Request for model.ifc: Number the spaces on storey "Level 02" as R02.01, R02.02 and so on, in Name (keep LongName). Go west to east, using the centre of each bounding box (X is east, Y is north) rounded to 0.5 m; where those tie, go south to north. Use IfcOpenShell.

First a look at what the model holds.

```python
import ifcopenshell
import ifcopenshell.util.element
import ifcopenshell.util.placement

model = ifcopenshell.open("model.ifc")
print(model.schema)
storey = next(s for s in model.by_type("IfcBuildingStorey") if s.Name == "Level 02")
spaces = [e for e in ifcopenshell.util.element.get_decomposition(storey) if e.is_a("IfcSpace")]
for e in sorted(spaces, key=lambda e: e.id()):
    origin = ifcopenshell.util.placement.get_local_placement(e.ObjectPlacement)[:3, 3]
    print(e.id(), e.Name, e.LongName, origin.round(2) + 0.0, sep=" | ")
```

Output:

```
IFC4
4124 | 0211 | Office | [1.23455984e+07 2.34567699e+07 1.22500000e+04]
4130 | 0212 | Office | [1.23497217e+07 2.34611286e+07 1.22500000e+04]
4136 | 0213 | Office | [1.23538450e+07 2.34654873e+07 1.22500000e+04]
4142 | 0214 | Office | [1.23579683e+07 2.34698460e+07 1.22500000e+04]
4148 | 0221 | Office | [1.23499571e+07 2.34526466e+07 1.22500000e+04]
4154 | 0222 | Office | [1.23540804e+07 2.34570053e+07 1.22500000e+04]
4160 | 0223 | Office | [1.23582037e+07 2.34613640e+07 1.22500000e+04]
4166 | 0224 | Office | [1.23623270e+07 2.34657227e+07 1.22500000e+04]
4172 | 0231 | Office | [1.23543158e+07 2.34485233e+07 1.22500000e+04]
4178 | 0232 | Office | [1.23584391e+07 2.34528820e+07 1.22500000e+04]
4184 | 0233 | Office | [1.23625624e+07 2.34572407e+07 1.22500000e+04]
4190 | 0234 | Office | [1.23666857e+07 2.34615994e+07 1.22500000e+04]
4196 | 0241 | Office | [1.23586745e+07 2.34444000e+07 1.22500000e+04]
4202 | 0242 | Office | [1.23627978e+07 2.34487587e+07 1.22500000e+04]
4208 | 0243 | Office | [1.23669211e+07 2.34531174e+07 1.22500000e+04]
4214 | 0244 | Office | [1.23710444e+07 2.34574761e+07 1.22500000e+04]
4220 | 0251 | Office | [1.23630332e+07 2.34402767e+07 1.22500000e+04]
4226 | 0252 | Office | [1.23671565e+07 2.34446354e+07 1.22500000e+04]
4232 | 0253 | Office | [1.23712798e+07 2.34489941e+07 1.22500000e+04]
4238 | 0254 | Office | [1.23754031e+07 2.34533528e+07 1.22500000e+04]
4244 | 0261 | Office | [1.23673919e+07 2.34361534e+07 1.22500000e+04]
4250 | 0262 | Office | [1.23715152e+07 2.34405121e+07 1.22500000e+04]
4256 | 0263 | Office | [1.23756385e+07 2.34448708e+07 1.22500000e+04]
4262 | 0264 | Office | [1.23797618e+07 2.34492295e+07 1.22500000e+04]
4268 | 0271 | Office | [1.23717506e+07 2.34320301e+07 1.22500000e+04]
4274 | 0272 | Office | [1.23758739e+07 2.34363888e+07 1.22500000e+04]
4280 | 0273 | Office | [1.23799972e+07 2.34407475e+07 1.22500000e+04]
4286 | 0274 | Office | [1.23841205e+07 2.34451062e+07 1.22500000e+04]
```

```python
import ifcopenshell
import ifcopenshell.geom
import ifcopenshell.util.element
import ifcopenshell.util.shape

model = ifcopenshell.open("model.ifc")
settings = ifcopenshell.geom.settings()
settings.set("use-world-coords", True)


def centre(element):
    shape = ifcopenshell.geom.create_shape(settings, element)
    return ifcopenshell.util.shape.get_bbox_centroid(shape.geometry)


storey = next(s for s in model.by_type("IfcBuildingStorey") if s.Name == "Level 02")
spaces = [e for e in ifcopenshell.util.element.get_decomposition(storey) if e.is_a("IfcSpace")]

# Insertion points can sit at a corner or the storey origin, so sort by the geometry (in metres).
centres = {e: centre(e) for e in spaces}
spaces.sort(key=lambda e: (round(centres[e][0] / 0.5), centres[e][1]))

for i, e in enumerate(spaces, start=1):
    number = f"R02.{i:02d}"
    e.Name = number
    print(e.id(), number)

model.write("model_v2.ifc")
```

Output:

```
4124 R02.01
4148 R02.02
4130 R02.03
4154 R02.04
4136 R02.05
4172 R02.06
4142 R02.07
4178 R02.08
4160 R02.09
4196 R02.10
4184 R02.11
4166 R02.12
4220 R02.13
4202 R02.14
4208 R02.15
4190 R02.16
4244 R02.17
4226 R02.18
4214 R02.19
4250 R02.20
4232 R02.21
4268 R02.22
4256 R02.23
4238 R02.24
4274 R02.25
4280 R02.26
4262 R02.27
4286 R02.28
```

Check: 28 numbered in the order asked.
